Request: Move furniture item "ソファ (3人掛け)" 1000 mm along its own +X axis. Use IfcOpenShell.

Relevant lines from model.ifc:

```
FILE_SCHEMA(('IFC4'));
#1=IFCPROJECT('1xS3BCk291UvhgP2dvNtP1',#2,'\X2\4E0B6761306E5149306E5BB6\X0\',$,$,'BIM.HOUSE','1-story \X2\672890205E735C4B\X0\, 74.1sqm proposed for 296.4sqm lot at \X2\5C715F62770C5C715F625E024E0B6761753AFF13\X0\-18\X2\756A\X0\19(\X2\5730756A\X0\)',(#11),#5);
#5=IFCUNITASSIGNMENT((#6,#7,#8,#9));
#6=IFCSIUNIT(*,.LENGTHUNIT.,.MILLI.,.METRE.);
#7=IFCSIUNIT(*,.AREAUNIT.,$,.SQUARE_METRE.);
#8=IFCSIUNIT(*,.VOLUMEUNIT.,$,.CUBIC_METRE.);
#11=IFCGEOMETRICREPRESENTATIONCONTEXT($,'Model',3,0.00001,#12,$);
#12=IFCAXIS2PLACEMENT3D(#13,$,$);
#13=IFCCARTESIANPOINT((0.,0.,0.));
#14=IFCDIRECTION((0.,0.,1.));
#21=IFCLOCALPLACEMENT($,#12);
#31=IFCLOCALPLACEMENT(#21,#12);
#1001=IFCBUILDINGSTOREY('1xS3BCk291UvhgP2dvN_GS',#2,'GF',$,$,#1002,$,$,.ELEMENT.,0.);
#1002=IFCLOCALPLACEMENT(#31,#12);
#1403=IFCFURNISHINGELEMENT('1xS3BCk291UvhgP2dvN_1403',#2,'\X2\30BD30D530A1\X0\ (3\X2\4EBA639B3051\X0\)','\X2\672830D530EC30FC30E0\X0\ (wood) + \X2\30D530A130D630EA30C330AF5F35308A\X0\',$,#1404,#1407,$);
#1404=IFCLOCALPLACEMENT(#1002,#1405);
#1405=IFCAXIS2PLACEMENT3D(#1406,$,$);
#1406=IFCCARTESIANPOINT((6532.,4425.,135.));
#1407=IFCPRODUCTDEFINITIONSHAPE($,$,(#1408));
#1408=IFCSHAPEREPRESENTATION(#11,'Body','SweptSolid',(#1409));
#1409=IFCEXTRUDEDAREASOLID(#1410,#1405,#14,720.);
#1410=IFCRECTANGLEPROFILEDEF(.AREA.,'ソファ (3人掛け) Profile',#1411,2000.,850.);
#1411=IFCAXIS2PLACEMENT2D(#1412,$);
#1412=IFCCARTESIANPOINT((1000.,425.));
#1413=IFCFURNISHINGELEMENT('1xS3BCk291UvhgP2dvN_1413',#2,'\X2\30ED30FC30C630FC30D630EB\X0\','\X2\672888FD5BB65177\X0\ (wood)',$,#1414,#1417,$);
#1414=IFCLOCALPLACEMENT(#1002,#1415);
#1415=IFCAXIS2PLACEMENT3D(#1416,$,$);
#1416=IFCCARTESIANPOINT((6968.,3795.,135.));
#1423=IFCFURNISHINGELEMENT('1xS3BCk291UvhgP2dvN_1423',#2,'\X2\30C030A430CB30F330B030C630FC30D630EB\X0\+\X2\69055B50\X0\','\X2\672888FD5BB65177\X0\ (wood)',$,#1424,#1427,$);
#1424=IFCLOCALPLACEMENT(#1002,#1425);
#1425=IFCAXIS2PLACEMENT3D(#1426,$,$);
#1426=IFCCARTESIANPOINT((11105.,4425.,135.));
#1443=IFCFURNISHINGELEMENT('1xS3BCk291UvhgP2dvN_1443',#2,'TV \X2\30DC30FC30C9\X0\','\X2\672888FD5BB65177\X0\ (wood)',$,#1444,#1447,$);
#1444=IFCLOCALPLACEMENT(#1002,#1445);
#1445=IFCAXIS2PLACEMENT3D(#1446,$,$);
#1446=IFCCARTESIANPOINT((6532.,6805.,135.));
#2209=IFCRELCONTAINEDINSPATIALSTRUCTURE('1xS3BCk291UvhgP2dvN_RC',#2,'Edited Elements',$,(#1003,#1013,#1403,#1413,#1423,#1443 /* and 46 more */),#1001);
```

```python
import ifcopenshell
import ifcopenshell.api.geometry
import ifcopenshell.util.placement
import ifcopenshell.util.unit

model = ifcopenshell.open("model.ifc")
unit_scale = ifcopenshell.util.unit.calculate_unit_scale(model)

item = model.by_guid("1xS3BCk291UvhgP2dvN_1403")
matrix = ifcopenshell.util.placement.get_local_placement(item.ObjectPlacement)
matrix[:3, 3] += matrix[:3, 0] * 1 / unit_scale
ifcopenshell.api.geometry.edit_object_placement(model, product=item, matrix=matrix, is_si=False)

print(ifcopenshell.util.placement.get_local_placement(item.ObjectPlacement).round(3) + 0.0)

model.write("model_edited.ifc")
```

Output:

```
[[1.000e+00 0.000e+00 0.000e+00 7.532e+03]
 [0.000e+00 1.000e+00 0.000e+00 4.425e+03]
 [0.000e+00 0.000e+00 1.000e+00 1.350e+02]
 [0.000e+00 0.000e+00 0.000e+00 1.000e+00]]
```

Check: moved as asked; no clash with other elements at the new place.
